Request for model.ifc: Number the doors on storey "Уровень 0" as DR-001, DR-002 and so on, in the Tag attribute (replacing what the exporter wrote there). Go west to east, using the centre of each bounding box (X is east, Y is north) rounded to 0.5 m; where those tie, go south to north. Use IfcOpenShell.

First a look at what the model holds.

```python
import ifcopenshell
import ifcopenshell.util.element
import ifcopenshell.util.placement

model = ifcopenshell.open("model.ifc")
print(model.schema)
storey = next(s for s in model.by_type("IfcBuildingStorey") if s.Name == "Уровень 0")
doors = [e for e in ifcopenshell.util.element.get_decomposition(storey) if e.is_a("IfcDoor")]
for e in sorted(doors, key=lambda e: e.id()):
    origin = ifcopenshell.util.placement.get_local_placement(e.ObjectPlacement)[:3, 3]
    print(e.id(), e.Tag, e.Name, origin.round(2) + 0.0, sep=" | ")
```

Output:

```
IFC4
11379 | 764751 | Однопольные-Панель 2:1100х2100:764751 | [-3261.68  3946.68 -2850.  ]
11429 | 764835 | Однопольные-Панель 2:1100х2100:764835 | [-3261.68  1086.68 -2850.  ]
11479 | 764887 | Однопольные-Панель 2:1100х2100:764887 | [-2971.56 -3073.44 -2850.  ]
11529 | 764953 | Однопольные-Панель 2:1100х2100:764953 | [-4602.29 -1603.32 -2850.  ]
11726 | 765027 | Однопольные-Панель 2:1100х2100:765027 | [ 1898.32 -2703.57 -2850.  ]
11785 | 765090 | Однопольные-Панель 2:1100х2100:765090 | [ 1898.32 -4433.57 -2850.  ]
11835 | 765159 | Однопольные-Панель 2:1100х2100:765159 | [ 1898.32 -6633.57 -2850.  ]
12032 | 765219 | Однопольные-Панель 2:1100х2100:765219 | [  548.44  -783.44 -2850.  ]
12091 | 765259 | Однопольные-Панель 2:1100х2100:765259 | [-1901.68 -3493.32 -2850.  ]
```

```python
import ifcopenshell
import ifcopenshell.geom
import ifcopenshell.util.element
import ifcopenshell.util.shape

model = ifcopenshell.open("model.ifc")
settings = ifcopenshell.geom.settings()
settings.set("use-world-coords", True)


def centre(element):
    shape = ifcopenshell.geom.create_shape(settings, element)
    return ifcopenshell.util.shape.get_bbox_centroid(shape.geometry)


storey = next(s for s in model.by_type("IfcBuildingStorey") if s.Name == "Уровень 0")
doors = [e for e in ifcopenshell.util.element.get_decomposition(storey) if e.is_a("IfcDoor")]

# Insertion points can sit at a corner or the storey origin, so sort by the geometry (in metres).
centres = {e: centre(e) for e in doors}
doors.sort(key=lambda e: (round(centres[e][0] / 0.5), centres[e][1]))

for i, e in enumerate(doors, start=1):
    number = f"DR-0{i:02d}"
    e.Tag = number
    print(e.id(), number)

model.write("model_updated.ifc")
```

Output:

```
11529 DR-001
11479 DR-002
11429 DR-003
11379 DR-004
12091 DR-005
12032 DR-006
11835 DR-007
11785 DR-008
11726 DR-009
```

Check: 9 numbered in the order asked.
